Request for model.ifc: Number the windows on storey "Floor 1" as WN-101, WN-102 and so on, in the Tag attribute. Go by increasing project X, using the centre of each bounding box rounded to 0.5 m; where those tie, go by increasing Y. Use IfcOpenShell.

First a look at what the model holds.

```python
import ifcopenshell
import ifcopenshell.util.element
import ifcopenshell.util.placement

model = ifcopenshell.open("model.ifc")
print(model.schema)
storey = next(s for s in model.by_type("IfcBuildingStorey") if s.Name == "Floor 1")
windows = [e for e in ifcopenshell.util.element.get_decomposition(storey) if e.is_a("IfcWindow")]
for e in sorted(windows, key=lambda e: e.id()):
    origin = ifcopenshell.util.placement.get_local_placement(e.ObjectPlacement)[:3, 3]
    print(e.id(), e.Tag, e.Name, origin.round(2) + 0.0, sep=" | ")
```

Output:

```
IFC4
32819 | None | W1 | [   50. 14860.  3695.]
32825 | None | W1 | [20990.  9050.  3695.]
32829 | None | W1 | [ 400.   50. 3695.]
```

```python
import ifcopenshell
import ifcopenshell.geom
import ifcopenshell.util.element
import ifcopenshell.util.shape

model = ifcopenshell.open("model.ifc")
settings = ifcopenshell.geom.settings()
settings.set("use-world-coords", True)


def centre(element):
    shape = ifcopenshell.geom.create_shape(settings, element)
    return ifcopenshell.util.shape.get_bbox_centroid(shape.geometry)


storey = next(s for s in model.by_type("IfcBuildingStorey") if s.Name == "Floor 1")
windows = [e for e in ifcopenshell.util.element.get_decomposition(storey) if e.is_a("IfcWindow")]

# Insertion points can sit at a corner or the storey origin, so sort by the geometry (in metres).
centres = {e: centre(e) for e in windows}
windows.sort(key=lambda e: (round(centres[e][0] / 0.5), centres[e][1]))

for i, e in enumerate(windows, start=1):
    number = f"WN-1{i:02d}"
    e.Tag = number
    print(e.id(), number)

model.write("model-out.ifc")
```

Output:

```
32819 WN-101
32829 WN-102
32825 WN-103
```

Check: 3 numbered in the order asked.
